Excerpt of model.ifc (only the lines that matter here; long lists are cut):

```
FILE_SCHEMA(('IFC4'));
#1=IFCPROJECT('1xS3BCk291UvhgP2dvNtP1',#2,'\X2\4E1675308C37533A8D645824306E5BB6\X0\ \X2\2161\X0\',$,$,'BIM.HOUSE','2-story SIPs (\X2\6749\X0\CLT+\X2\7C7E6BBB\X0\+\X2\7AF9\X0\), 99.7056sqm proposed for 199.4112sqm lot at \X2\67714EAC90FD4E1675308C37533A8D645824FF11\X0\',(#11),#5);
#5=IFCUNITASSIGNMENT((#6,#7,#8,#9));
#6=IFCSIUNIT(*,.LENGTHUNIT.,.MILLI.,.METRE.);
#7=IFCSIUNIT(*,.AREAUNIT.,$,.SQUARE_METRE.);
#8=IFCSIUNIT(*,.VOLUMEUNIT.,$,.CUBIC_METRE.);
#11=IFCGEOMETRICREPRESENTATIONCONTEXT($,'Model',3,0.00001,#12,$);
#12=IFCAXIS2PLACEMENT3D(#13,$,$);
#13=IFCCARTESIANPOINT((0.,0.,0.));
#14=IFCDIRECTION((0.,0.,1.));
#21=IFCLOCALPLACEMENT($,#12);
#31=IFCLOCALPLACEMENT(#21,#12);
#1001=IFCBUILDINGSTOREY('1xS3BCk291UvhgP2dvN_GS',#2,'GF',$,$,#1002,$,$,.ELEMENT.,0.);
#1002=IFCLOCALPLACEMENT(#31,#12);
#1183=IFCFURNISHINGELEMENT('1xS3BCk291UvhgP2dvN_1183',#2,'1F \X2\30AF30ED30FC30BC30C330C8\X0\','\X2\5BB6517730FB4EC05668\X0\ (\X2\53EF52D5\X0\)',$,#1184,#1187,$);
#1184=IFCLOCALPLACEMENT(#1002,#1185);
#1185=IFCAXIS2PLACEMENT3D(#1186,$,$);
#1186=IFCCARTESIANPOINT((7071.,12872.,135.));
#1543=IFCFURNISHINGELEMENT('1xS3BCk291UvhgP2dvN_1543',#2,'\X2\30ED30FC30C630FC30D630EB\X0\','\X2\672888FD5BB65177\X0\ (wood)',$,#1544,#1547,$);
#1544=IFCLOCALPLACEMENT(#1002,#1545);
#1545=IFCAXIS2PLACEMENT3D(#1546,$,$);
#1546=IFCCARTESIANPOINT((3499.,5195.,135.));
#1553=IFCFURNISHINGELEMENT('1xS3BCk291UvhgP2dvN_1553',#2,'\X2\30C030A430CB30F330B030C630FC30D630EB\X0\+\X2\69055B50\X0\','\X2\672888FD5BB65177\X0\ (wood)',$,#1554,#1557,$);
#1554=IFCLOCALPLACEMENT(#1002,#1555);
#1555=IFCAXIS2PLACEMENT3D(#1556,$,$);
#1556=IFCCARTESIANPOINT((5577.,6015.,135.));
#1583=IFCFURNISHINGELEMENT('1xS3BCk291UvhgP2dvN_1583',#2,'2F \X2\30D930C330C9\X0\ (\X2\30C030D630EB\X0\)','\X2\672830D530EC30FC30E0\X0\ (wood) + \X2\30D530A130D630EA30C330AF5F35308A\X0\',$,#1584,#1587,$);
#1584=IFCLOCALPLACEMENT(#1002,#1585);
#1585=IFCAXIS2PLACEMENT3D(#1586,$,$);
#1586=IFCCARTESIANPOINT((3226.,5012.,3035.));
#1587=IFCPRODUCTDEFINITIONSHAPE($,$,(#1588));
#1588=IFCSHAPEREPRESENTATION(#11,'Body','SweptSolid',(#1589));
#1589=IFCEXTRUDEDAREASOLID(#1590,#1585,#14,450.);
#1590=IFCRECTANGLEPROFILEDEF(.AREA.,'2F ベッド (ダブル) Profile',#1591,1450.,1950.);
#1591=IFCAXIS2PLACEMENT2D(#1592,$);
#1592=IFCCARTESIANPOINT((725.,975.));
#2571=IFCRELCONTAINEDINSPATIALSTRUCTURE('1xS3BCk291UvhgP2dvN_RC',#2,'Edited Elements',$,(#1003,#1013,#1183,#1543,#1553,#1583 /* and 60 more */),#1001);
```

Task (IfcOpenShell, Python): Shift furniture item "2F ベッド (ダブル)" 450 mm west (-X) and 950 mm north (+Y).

```python
import ifcopenshell
import ifcopenshell.api.geometry
import ifcopenshell.util.placement
import ifcopenshell.util.unit

model = ifcopenshell.open("model.ifc")
unit_scale = ifcopenshell.util.unit.calculate_unit_scale(model)

item = model.by_guid("1xS3BCk291UvhgP2dvN_1583")
matrix = ifcopenshell.util.placement.get_local_placement(item.ObjectPlacement)
matrix[0, 3] -= 0.45 / unit_scale
matrix[1, 3] += 0.95 / unit_scale
ifcopenshell.api.geometry.edit_object_placement(model, product=item, matrix=matrix, is_si=False)

print(ifcopenshell.util.placement.get_local_placement(item.ObjectPlacement).round(3) + 0.0)

model.write("model-out.ifc")
```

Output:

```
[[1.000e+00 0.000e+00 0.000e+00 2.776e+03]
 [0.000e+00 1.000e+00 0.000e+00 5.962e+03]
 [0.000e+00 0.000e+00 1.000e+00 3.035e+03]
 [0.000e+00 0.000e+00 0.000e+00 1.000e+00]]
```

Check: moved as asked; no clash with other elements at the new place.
